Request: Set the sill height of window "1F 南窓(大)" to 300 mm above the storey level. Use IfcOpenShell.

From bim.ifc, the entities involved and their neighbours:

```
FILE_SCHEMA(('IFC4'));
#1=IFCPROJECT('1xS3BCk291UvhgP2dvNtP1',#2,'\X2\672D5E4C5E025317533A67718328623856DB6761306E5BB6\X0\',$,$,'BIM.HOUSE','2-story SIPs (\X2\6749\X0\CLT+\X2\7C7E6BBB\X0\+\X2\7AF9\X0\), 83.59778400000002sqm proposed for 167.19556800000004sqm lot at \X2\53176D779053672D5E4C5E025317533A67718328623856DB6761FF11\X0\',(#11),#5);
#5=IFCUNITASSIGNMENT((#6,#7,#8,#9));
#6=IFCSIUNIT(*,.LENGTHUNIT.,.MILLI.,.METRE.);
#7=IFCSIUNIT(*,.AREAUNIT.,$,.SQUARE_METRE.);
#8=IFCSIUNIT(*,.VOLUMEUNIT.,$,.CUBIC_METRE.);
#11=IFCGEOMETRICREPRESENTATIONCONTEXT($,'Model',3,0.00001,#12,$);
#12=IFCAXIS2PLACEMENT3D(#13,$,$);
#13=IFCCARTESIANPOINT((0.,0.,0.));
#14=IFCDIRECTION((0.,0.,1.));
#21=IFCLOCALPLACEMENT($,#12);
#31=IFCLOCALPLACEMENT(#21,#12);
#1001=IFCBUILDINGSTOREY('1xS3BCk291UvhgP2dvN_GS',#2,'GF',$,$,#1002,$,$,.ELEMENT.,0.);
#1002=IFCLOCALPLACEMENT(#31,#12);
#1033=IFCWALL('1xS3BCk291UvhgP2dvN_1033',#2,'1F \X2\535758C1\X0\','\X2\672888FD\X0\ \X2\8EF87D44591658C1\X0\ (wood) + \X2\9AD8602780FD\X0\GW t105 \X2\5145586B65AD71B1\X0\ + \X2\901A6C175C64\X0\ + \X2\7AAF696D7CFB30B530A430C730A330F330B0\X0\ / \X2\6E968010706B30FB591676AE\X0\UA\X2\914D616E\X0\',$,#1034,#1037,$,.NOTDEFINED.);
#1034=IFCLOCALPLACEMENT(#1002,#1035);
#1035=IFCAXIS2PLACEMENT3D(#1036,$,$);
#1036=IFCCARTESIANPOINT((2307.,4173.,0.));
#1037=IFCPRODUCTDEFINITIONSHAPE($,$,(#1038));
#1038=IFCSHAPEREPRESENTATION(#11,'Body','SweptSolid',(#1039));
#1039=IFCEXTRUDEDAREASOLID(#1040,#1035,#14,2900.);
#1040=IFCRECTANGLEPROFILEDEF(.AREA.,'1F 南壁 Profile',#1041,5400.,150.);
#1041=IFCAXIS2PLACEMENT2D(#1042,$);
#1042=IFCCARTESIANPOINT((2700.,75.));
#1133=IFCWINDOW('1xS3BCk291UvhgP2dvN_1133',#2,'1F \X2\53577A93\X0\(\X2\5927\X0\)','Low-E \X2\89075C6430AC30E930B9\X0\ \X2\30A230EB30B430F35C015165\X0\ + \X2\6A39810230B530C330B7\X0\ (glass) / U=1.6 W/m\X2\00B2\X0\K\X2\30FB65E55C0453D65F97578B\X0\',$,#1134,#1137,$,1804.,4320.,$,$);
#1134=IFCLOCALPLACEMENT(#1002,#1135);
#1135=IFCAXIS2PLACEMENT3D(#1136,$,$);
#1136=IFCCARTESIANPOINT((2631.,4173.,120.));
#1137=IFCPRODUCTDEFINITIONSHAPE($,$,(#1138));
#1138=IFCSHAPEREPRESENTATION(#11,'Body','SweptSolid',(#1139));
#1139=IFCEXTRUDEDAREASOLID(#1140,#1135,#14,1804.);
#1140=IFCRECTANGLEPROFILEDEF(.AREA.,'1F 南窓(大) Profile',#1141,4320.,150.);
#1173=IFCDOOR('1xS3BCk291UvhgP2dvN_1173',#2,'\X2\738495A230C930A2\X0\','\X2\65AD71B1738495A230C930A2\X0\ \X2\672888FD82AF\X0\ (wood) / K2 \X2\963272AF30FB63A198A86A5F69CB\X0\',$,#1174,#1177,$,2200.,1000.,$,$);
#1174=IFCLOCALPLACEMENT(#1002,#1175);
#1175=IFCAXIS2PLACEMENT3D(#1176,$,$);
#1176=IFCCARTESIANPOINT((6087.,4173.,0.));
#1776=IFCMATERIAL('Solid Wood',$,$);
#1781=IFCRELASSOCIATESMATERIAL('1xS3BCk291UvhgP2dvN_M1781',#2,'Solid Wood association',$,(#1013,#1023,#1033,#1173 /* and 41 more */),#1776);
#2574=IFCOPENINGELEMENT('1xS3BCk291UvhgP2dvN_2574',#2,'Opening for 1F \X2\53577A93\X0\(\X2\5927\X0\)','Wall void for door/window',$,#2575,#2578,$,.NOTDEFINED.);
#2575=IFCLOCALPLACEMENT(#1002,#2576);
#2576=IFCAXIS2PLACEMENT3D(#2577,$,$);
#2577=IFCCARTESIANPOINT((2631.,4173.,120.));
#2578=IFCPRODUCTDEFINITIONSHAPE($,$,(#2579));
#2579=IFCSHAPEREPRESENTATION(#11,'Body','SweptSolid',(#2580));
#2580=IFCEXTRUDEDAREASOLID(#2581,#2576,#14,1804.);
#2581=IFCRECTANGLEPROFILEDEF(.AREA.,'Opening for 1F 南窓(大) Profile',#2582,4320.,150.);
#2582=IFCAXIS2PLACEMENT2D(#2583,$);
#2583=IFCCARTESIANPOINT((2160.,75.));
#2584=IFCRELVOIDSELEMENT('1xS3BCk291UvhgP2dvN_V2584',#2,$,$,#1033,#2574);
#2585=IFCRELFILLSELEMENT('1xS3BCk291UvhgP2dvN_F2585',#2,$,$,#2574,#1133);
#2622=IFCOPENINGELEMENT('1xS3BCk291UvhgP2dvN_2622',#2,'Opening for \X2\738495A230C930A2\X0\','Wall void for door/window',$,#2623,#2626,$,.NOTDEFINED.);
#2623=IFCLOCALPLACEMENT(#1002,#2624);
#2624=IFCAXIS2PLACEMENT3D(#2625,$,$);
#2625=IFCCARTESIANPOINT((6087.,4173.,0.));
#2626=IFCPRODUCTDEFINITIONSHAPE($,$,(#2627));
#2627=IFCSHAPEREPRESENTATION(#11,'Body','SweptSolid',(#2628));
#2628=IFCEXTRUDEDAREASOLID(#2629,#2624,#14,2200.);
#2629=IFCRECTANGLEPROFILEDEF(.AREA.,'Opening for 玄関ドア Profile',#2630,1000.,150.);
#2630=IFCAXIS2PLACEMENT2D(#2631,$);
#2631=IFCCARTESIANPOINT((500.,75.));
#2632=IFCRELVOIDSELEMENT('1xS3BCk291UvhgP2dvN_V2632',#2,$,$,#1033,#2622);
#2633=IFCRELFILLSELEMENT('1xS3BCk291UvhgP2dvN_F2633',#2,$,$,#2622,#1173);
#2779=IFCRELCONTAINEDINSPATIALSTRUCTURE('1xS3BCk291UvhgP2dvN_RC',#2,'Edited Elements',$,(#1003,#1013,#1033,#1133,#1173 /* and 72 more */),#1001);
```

```python
import numpy as np
import ifcopenshell
import ifcopenshell.api.geometry
import ifcopenshell.geom
import ifcopenshell.util.element
import ifcopenshell.util.placement
import ifcopenshell.util.shape
import ifcopenshell.util.unit

model = ifcopenshell.open("bim.ifc")
unit_scale = ifcopenshell.util.unit.calculate_unit_scale(model)

window = model.by_id(1133)
opening = window.FillsVoids[0].RelatingOpeningElement
storey = ifcopenshell.util.element.get_container(window, ifc_class="IfcBuildingStorey")
level = ifcopenshell.util.placement.get_local_placement(storey.ObjectPlacement)[2, 3]

# The opening's origin need not be at the sill, so measure its lowest point.
shape = ifcopenshell.geom.create_shape(ifcopenshell.geom.settings(), opening)
bottom = ifcopenshell.util.shape.get_shape_bottom_elevation(shape, shape.geometry) / unit_scale
dz = level + 300.0 - bottom

shift = np.array([0.0, 0.0, dz])
# The window is not placed relative to its opening, so move both.
for product in (opening, window):
    matrix = ifcopenshell.util.placement.get_local_placement(product.ObjectPlacement)
    matrix[:3, 3] += shift
    ifcopenshell.api.geometry.edit_object_placement(model, product=product, matrix=matrix, is_si=False)

print(f"moved by {dz * unit_scale:+.3f} m")

model.write("bim_edited.ifc")
```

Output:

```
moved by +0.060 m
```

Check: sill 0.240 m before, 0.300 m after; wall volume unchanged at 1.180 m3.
